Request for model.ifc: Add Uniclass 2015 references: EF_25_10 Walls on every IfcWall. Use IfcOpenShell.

First a look at what the model holds.

```python
import ifcopenshell

model = ifcopenshell.open("model.ifc")
print(model.schema)
print("classifications:", [c.Name for c in model.by_type("IfcClassification")])
for ifc_class in ("IfcDoor", "IfcRoof", "IfcStair", "IfcWall", "IfcWindow"):
    print(ifc_class, len(model.by_type(ifc_class)))
```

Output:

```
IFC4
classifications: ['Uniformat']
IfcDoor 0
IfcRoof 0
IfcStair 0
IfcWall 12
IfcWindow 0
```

```python
import ifcopenshell
import ifcopenshell.api.classification

model = ifcopenshell.open("model.ifc")

system = ifcopenshell.api.classification.add_classification(model, classification="Uniclass 2015")

codes = {
    "IfcWall": ("EF_25_10", "Walls"),
}
for ifc_class, (code, name) in codes.items():
    products = model.by_type(ifc_class)
    ifcopenshell.api.classification.add_reference(
        model, products=products, classification=system, identification=code, name=name
    )
    print(code, len(products))

model.write("model-out.ifc")
```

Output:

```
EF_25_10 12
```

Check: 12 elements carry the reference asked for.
